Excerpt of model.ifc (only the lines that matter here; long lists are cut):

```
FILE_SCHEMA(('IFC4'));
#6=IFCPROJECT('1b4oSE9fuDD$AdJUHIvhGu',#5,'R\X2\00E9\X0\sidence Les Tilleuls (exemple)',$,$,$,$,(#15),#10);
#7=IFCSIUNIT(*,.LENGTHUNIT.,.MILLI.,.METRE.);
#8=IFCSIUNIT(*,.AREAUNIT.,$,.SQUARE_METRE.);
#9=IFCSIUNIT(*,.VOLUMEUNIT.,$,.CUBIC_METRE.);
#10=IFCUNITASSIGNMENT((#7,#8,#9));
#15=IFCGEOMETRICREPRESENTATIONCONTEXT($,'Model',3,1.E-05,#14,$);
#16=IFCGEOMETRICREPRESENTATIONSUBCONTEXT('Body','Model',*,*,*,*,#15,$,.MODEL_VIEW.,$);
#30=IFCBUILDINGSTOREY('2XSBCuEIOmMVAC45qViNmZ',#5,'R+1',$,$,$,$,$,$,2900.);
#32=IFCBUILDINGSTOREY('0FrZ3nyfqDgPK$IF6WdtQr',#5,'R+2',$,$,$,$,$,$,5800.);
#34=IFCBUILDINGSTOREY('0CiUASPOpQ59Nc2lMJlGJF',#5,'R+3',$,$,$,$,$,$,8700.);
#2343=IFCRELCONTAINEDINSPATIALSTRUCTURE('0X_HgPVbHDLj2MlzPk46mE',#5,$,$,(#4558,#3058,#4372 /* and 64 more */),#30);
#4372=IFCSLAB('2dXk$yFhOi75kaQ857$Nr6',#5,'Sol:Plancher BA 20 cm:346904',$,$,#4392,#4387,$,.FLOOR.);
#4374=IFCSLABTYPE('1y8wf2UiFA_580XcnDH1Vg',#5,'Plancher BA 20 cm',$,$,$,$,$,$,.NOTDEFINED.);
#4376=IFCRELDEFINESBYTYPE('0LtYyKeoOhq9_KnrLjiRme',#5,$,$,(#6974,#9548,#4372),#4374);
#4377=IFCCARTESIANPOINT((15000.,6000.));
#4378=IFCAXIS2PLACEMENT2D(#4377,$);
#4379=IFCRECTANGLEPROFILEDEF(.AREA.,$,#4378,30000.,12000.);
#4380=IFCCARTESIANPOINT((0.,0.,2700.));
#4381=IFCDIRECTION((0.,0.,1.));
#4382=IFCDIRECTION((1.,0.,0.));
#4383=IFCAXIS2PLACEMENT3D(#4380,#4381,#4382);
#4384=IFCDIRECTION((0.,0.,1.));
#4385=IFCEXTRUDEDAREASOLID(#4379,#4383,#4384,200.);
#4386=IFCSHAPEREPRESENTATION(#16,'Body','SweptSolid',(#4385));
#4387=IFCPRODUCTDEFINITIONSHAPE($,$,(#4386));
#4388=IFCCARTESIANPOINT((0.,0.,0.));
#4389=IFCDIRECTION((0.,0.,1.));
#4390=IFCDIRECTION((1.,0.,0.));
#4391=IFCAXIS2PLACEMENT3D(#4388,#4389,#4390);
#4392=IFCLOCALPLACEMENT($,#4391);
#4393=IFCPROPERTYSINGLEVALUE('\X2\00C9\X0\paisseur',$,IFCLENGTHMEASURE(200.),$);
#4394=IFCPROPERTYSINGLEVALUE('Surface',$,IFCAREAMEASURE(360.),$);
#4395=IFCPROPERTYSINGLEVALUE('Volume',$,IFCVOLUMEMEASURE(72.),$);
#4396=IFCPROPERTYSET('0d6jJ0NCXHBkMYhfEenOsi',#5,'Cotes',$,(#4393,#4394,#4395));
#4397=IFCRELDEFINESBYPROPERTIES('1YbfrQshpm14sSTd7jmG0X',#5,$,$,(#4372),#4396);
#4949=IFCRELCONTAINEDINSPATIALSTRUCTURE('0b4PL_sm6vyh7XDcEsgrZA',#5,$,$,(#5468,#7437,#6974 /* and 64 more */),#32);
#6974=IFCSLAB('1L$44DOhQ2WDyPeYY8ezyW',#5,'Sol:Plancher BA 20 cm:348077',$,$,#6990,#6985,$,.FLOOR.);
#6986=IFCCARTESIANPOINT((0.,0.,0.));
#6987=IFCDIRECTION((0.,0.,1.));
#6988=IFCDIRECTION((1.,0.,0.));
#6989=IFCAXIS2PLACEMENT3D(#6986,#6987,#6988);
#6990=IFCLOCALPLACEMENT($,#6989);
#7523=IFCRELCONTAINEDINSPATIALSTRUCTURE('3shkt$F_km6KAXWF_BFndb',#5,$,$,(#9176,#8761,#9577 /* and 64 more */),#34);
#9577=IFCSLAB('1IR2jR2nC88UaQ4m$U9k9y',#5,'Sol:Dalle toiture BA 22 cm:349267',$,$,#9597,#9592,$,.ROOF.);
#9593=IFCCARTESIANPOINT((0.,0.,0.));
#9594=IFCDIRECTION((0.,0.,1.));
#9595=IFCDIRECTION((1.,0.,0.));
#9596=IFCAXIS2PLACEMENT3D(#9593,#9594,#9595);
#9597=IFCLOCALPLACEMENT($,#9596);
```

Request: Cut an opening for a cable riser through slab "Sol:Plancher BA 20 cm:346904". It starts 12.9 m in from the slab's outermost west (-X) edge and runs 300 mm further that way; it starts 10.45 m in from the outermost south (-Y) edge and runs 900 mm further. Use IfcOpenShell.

```python
import numpy as np
import ifcopenshell
import ifcopenshell.api.feature
import ifcopenshell.api.geometry
import ifcopenshell.api.pset
import ifcopenshell.api.root
import ifcopenshell.geom
import ifcopenshell.util.element
import ifcopenshell.util.placement
import ifcopenshell.util.representation
import ifcopenshell.util.shape
import ifcopenshell.util.unit

model = ifcopenshell.open("model.ifc")
unit_scale = ifcopenshell.util.unit.calculate_unit_scale(model)
area_scale = ifcopenshell.util.unit.calculate_unit_scale(model, "AREAUNIT")
volume_scale = ifcopenshell.util.unit.calculate_unit_scale(model, "VOLUMEUNIT")
settings = ifcopenshell.geom.settings()


def volume(element):
    """Net volume in cubic metres, openings subtracted."""
    shape = ifcopenshell.geom.create_shape(settings, element)
    return ifcopenshell.util.shape.get_volume(shape.geometry)


slab = model.by_guid("2dXk$yFhOi75kaQ857$Nr6")
before = volume(slab)

# Extent in the slab's own axes, in metres. The edges named are its -X and -Y sides.
slab_shape = ifcopenshell.geom.create_shape(settings, slab)
vertices = ifcopenshell.util.shape.get_vertices(slab_shape.geometry)
x_min, y_min, bottom = vertices.min(axis=0)
top = vertices[:, 2].max()

opening = ifcopenshell.api.root.create_entity(model, ifc_class="IfcOpeningElement", name="Cable riser opening", predefined_type="OPENING")
context = ifcopenshell.util.representation.get_context(model, "Model", "Body", "MODEL_VIEW")
width, depth = 0.3, 0.9
outline = [(0.0, 0.0), (width, 0.0), (width, depth), (0.0, depth), (0.0, 0.0)]
# Overshoot both faces by 50 mm so the cut is clean.
shape = ifcopenshell.api.geometry.add_slab_representation(
    model, context=context, depth=top - bottom + 0.1, polyline=outline
)
ifcopenshell.api.geometry.assign_representation(model, product=opening, representation=shape)

matrix = ifcopenshell.util.placement.get_local_placement(slab.ObjectPlacement)
matrix[:, 3] = matrix @ np.append(np.array([x_min + 12.9, y_min + 10.45, bottom - 0.05]) / unit_scale, 1.0)
ifcopenshell.api.geometry.edit_object_placement(model, product=opening, matrix=matrix, is_si=False)
ifcopenshell.api.feature.add_feature(model, feature=opening, element=slab)

after = volume(slab)

# Update the slab's stored quantities.
pset = model.by_id(ifcopenshell.util.element.get_pset(slab, "Cotes", should_inherit=False)["id"])
ifcopenshell.api.pset.edit_pset(model, pset=pset, properties={
    "Surface": model.create_entity("IfcAreaMeasure", after / (top - bottom) / area_scale),
    "Volume": model.create_entity("IfcVolumeMeasure", after / volume_scale),
})

print(f"slab volume {before:.3f} -> {after:.3f} m3")

model.write("model_updated.ifc")
```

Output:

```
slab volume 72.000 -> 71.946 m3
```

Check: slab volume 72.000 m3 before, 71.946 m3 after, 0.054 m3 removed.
